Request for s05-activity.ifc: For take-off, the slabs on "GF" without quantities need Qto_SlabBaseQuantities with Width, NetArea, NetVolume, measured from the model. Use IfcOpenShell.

First a look at what the model holds.

```python
import ifcopenshell
import ifcopenshell.util.element
import ifcopenshell.util.unit

model = ifcopenshell.open("s05-activity.ifc")
print(model.schema)
for unit_type in ("LENGTHUNIT", "AREAUNIT", "VOLUMEUNIT"):
    print(unit_type, ifcopenshell.util.unit.calculate_unit_scale(model, unit_type))
storey = next(s for s in model.by_type("IfcBuildingStorey") if s.Name == "GF")
slabs = [e for e in ifcopenshell.util.element.get_decomposition(storey) if e.is_a("IfcSlab")]
for e in sorted(slabs, key=lambda e: e.id()):
    print(e.id(), e.is_a(), e.Name, list(ifcopenshell.util.element.get_psets(e, qtos_only=True)), sep=" | ")
```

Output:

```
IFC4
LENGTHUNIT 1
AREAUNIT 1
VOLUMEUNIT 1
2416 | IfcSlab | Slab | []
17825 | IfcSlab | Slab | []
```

```python
import ifcopenshell
import ifcopenshell.api.pset
import ifcopenshell.geom
import ifcopenshell.util.element
import ifcopenshell.util.shape
import ifcopenshell.util.unit

model = ifcopenshell.open("s05-activity.ifc")
unit_scale = ifcopenshell.util.unit.calculate_unit_scale(model)
area_scale = ifcopenshell.util.unit.calculate_unit_scale(model, "AREAUNIT")
volume_scale = ifcopenshell.util.unit.calculate_unit_scale(model, "VOLUMEUNIT")
settings = ifcopenshell.geom.settings()

storey = next(s for s in model.by_type("IfcBuildingStorey") if s.Name == "GF")
slabs = [e for e in ifcopenshell.util.element.get_decomposition(storey) if e.is_a("IfcSlab")]

for e in sorted(slabs, key=lambda e: e.id()):
    if ifcopenshell.util.element.get_psets(e, qtos_only=True, should_inherit=False):
        continue
    # Geometry comes back in metres, in the element's own axes.
    shape = ifcopenshell.geom.create_shape(settings, e)
    values = {
        "Width": ifcopenshell.util.shape.get_z(shape.geometry) / unit_scale,
        "NetArea": ifcopenshell.util.shape.get_footprint_area(shape.geometry) / area_scale,
        "NetVolume": ifcopenshell.util.shape.get_volume(shape.geometry) / volume_scale,
    }
    qto = ifcopenshell.api.pset.add_qto(model, product=e, name="Qto_SlabBaseQuantities")
    ifcopenshell.api.pset.edit_qto(model, qto=qto, properties=values)
    print(e.id(), {k: round(v, 3) for k, v in values.items()})

model.write("s05-activity_rev.ifc")
```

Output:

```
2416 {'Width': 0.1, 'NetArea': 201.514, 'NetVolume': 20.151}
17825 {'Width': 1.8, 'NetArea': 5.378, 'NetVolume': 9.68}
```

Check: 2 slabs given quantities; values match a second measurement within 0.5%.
